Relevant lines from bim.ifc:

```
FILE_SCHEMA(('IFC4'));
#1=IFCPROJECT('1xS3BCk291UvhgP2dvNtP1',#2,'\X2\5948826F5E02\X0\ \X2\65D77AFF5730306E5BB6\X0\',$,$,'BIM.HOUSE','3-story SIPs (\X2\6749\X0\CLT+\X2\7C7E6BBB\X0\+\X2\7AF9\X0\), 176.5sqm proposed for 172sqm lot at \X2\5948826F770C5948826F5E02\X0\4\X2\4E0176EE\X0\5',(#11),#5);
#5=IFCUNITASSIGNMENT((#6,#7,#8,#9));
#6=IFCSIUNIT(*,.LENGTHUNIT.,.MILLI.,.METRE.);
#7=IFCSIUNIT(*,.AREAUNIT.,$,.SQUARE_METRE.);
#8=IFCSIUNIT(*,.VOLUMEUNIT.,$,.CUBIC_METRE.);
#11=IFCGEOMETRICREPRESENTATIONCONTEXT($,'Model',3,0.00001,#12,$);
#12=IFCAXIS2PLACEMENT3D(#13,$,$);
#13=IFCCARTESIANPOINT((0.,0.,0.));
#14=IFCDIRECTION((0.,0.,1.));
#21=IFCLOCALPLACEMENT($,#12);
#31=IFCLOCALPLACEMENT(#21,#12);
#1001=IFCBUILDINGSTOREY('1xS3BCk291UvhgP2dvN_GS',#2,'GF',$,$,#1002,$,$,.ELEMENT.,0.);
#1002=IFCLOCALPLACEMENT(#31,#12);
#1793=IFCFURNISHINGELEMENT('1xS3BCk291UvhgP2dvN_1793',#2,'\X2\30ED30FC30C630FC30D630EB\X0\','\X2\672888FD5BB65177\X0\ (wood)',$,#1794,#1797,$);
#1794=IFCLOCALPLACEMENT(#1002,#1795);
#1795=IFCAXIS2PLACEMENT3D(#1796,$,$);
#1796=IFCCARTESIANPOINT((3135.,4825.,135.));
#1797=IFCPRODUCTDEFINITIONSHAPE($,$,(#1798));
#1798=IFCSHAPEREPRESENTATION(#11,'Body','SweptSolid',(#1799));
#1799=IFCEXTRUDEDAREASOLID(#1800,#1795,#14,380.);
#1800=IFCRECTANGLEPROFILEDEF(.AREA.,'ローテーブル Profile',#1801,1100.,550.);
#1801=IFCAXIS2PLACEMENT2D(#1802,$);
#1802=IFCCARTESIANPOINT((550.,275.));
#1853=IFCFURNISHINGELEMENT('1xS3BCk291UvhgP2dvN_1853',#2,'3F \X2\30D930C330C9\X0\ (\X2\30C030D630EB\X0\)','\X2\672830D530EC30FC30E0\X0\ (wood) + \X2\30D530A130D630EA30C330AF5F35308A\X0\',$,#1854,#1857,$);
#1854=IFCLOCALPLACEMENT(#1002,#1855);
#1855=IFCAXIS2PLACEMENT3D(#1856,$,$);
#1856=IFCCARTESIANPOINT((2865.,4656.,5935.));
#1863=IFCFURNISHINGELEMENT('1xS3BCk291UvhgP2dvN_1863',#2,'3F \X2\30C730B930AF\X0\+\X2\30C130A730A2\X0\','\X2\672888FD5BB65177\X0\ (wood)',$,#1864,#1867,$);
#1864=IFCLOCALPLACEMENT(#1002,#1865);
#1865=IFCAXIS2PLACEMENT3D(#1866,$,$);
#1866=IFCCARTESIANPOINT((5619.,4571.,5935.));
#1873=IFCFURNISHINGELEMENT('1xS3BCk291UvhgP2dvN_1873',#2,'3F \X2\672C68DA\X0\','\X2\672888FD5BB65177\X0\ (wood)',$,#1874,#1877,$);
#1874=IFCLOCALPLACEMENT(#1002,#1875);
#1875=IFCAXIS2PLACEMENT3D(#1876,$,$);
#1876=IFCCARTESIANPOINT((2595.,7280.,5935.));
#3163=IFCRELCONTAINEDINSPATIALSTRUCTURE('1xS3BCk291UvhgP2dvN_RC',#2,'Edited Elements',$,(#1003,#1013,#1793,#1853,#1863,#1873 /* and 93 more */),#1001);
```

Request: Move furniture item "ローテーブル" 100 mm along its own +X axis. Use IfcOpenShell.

```python
import ifcopenshell
import ifcopenshell.api.geometry
import ifcopenshell.util.placement
import ifcopenshell.util.unit

model = ifcopenshell.open("bim.ifc")
unit_scale = ifcopenshell.util.unit.calculate_unit_scale(model)

item = model.by_guid("1xS3BCk291UvhgP2dvN_1793")
matrix = ifcopenshell.util.placement.get_local_placement(item.ObjectPlacement)
matrix[:3, 3] += matrix[:3, 0] * 0.1 / unit_scale
ifcopenshell.api.geometry.edit_object_placement(model, product=item, matrix=matrix, is_si=False)

print(ifcopenshell.util.placement.get_local_placement(item.ObjectPlacement).round(3) + 0.0)

model.write("bim_edited.ifc")
```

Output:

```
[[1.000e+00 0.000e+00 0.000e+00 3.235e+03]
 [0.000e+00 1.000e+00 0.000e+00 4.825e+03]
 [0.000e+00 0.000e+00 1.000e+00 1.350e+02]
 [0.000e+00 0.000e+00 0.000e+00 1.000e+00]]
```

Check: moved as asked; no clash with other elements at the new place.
